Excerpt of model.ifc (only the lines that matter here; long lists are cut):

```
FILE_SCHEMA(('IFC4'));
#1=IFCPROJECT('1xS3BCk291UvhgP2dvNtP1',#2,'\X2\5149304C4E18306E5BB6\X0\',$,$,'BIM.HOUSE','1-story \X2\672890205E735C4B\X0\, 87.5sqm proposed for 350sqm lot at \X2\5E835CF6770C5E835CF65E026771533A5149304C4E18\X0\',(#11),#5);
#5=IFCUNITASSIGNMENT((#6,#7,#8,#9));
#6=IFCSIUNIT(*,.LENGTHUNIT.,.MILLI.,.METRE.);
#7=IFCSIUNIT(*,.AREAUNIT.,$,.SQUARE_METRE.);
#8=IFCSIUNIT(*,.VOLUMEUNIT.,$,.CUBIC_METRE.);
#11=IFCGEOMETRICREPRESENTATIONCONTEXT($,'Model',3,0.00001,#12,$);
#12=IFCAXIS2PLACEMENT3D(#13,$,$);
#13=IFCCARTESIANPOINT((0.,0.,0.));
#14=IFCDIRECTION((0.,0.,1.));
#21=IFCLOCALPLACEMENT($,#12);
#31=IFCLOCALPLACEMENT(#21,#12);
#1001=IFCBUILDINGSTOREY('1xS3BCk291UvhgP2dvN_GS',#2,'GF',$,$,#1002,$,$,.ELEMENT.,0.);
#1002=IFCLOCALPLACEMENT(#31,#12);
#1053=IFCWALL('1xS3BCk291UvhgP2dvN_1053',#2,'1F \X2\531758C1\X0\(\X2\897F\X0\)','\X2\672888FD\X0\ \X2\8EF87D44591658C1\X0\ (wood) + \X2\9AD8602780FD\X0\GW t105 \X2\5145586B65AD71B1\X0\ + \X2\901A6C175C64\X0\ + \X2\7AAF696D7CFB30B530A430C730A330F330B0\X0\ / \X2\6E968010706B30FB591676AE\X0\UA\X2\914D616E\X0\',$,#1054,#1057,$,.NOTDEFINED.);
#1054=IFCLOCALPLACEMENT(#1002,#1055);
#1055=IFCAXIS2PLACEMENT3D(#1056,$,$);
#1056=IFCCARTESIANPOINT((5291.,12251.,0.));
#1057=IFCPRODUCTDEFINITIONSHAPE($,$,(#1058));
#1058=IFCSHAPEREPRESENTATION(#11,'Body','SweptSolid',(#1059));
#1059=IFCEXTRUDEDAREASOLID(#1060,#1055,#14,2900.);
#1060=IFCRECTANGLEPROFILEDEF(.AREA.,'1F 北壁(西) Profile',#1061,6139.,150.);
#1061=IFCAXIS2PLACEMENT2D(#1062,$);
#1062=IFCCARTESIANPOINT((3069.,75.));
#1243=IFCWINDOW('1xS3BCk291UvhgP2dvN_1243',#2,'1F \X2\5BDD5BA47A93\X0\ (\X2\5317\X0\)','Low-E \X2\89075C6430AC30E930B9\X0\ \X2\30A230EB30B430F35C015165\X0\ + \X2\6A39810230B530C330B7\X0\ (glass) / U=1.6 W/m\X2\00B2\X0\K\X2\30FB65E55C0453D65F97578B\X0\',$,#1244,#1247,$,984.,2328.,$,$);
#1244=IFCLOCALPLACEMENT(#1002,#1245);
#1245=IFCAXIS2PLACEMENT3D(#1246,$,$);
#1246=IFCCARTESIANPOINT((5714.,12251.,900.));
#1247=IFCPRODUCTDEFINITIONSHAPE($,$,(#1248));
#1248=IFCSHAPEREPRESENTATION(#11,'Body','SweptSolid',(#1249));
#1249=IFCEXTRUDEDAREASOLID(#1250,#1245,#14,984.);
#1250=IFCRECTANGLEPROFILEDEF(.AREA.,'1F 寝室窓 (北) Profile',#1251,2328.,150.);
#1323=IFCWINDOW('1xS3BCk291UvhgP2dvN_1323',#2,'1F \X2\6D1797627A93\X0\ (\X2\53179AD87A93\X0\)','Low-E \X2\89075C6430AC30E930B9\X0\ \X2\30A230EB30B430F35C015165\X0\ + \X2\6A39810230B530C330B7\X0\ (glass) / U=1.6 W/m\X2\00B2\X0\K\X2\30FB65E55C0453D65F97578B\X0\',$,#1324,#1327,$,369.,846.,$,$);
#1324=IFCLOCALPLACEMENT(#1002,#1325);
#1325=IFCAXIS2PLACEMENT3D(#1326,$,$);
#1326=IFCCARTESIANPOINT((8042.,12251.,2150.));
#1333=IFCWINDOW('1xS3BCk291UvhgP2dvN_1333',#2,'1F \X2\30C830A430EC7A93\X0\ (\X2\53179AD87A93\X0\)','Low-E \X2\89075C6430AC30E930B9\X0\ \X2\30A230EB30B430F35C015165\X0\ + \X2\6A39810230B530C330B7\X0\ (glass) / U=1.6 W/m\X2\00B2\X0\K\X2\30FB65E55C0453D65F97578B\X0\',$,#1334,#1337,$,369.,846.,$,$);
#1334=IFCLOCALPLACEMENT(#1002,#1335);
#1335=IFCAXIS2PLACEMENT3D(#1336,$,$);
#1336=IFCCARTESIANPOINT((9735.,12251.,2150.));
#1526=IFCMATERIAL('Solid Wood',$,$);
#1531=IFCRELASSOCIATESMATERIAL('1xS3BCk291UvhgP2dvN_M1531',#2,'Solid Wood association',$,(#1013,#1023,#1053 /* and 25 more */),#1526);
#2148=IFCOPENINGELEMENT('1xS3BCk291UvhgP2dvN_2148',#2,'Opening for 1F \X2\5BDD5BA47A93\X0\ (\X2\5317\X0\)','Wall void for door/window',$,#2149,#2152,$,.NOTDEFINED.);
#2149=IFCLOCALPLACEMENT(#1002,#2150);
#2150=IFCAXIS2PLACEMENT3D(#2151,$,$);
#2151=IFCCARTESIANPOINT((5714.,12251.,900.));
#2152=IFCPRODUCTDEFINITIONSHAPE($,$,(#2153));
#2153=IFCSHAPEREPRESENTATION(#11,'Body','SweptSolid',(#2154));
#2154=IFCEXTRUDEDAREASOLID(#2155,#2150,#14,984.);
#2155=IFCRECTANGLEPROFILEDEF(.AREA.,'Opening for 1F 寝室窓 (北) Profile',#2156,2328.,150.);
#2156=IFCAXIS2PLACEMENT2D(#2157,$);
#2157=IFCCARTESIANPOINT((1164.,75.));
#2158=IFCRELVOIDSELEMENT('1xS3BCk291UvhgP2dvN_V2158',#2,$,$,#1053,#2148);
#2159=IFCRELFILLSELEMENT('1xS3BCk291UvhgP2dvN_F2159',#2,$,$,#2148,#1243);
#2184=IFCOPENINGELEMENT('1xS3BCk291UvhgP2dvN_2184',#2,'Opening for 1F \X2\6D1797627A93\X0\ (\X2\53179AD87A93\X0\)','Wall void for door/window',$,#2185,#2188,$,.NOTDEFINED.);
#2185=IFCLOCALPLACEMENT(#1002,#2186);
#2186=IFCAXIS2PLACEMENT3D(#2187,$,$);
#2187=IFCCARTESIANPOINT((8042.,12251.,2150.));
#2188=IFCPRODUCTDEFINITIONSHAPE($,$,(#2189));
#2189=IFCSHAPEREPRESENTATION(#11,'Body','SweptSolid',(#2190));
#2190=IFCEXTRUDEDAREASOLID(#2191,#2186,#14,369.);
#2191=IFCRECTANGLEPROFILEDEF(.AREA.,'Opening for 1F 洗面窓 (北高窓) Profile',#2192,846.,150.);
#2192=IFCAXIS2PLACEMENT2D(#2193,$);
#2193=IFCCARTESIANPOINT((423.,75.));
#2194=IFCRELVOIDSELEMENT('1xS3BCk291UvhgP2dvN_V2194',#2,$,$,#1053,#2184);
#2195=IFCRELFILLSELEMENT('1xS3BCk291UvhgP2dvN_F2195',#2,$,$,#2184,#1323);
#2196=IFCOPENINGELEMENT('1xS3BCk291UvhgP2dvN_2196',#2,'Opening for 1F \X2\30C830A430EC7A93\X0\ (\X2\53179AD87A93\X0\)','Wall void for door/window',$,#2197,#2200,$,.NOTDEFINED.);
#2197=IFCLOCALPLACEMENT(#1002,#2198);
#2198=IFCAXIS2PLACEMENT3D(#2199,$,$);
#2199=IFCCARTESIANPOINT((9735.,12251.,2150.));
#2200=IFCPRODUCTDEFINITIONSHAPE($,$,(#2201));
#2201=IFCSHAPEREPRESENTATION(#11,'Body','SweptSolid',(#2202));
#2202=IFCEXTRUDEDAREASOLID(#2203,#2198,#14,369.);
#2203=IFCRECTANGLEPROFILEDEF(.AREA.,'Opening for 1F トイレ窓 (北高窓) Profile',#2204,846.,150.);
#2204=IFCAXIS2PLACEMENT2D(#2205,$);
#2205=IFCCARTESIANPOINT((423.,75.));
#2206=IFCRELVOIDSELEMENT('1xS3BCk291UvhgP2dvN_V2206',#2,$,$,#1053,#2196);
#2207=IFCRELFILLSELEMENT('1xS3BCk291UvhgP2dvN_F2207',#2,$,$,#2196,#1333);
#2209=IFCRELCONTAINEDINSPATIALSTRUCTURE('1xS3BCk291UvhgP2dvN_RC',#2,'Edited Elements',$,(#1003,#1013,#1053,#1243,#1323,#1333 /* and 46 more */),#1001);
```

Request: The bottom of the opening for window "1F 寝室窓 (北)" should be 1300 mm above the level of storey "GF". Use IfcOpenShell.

```python
import numpy as np
import ifcopenshell
import ifcopenshell.api.geometry
import ifcopenshell.geom
import ifcopenshell.util.element
import ifcopenshell.util.placement
import ifcopenshell.util.shape
import ifcopenshell.util.unit

model = ifcopenshell.open("model.ifc")
unit_scale = ifcopenshell.util.unit.calculate_unit_scale(model)

window = model.by_guid("1xS3BCk291UvhgP2dvN_1243")
opening = window.FillsVoids[0].RelatingOpeningElement
storey = ifcopenshell.util.element.get_container(window, ifc_class="IfcBuildingStorey")
level = ifcopenshell.util.placement.get_local_placement(storey.ObjectPlacement)[2, 3]

# The opening's origin need not be at the sill, so measure its lowest point.
shape = ifcopenshell.geom.create_shape(ifcopenshell.geom.settings(), opening)
bottom = ifcopenshell.util.shape.get_shape_bottom_elevation(shape, shape.geometry) / unit_scale
dz = level + 1300.0 - bottom

shift = np.array([0.0, 0.0, dz])
# The window is not placed relative to its opening, so move both.
for product in (opening, window):
    matrix = ifcopenshell.util.placement.get_local_placement(product.ObjectPlacement)
    matrix[:3, 3] += shift
    ifcopenshell.api.geometry.edit_object_placement(model, product=product, matrix=matrix, is_si=False)

print(f"moved by {dz * unit_scale:+.3f} m")

model.write("model_updated.ifc")
```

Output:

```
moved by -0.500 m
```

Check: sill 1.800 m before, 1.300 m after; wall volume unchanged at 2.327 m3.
